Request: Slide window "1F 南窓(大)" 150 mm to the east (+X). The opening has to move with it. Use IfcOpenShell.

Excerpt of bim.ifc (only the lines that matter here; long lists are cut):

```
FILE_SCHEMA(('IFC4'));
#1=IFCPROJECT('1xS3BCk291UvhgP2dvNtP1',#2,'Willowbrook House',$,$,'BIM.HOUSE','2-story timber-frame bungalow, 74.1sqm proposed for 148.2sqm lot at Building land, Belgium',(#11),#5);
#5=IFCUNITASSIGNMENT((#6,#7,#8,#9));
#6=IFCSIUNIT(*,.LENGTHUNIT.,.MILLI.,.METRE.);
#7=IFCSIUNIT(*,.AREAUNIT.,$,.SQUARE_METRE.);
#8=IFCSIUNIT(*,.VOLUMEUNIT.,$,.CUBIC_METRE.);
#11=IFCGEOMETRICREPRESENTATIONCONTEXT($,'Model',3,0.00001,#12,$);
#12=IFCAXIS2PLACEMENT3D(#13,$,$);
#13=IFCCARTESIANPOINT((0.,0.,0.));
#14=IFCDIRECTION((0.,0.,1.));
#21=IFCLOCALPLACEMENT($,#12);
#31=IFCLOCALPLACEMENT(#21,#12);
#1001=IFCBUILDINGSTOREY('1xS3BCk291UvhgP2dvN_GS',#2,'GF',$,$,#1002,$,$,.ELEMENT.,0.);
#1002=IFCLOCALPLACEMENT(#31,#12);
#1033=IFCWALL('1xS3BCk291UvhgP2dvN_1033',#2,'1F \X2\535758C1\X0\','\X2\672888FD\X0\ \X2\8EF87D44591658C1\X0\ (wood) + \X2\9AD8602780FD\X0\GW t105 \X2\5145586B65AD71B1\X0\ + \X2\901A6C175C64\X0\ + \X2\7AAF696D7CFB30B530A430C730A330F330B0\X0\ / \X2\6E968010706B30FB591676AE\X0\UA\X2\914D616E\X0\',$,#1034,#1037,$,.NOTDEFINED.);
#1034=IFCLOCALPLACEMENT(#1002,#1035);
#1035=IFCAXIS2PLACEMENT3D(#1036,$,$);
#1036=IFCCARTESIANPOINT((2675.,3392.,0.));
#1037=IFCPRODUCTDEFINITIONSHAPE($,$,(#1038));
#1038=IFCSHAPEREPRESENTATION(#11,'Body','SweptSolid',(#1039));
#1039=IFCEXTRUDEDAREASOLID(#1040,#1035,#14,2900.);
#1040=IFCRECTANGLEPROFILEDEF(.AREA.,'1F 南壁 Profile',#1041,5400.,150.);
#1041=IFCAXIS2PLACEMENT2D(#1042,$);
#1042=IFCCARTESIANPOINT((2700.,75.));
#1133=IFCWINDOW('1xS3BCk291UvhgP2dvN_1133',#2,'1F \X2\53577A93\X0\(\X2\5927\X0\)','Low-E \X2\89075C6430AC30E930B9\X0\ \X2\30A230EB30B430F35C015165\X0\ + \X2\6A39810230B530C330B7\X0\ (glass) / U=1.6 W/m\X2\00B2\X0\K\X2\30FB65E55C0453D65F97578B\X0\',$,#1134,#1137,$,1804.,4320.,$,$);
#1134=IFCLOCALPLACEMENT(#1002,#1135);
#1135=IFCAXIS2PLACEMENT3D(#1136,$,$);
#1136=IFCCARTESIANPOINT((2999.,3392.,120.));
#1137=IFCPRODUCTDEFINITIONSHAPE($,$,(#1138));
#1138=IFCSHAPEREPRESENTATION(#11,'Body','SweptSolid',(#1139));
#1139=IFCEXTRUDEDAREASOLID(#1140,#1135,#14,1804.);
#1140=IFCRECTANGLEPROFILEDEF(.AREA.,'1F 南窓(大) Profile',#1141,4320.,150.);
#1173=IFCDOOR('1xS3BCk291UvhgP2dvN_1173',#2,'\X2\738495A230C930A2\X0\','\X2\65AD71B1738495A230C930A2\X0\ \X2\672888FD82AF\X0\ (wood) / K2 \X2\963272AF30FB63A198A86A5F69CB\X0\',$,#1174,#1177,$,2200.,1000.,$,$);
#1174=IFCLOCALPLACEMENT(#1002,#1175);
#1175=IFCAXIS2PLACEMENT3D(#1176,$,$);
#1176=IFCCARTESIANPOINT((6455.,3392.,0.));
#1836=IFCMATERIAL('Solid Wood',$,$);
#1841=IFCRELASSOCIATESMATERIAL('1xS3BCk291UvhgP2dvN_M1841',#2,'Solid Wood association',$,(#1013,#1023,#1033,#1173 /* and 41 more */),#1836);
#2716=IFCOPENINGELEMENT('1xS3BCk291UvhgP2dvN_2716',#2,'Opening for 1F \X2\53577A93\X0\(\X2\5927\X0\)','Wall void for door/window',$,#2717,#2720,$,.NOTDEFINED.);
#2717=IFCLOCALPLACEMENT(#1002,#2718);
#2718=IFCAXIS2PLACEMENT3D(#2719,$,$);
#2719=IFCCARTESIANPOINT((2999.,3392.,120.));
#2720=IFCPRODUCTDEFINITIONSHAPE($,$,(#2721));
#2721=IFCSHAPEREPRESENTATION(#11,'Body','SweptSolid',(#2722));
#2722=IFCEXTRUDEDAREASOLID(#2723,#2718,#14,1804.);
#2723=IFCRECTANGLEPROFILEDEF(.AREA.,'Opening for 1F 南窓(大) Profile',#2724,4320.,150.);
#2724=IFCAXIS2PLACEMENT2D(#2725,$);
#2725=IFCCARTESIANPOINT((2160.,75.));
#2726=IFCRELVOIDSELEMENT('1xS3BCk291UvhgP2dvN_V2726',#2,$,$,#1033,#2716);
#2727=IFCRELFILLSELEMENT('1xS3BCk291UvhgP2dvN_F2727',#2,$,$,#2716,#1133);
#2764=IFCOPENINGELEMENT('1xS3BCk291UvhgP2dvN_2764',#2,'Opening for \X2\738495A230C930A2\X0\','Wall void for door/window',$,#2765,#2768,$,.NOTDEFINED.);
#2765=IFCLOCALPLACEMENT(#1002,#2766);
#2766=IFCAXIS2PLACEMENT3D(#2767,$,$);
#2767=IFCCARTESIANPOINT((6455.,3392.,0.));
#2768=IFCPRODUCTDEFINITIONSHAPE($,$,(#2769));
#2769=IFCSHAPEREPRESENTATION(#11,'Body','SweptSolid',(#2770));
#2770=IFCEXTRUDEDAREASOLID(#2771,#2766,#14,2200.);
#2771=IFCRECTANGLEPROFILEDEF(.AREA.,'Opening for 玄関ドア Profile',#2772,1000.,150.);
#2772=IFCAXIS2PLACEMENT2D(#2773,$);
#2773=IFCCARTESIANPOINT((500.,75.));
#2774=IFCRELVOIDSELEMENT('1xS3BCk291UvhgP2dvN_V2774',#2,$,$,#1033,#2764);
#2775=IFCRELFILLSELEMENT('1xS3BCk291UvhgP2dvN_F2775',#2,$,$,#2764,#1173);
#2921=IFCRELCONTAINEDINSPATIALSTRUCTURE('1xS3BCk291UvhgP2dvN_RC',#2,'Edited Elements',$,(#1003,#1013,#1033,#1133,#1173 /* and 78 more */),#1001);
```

```python
import ifcopenshell
import ifcopenshell.api.geometry
import ifcopenshell.util.placement
import ifcopenshell.util.unit

model = ifcopenshell.open("bim.ifc")
unit_scale = ifcopenshell.util.unit.calculate_unit_scale(model)

window = model.by_guid("1xS3BCk291UvhgP2dvN_1133")
opening = window.FillsVoids[0].RelatingOpeningElement
wall = opening.VoidsElements[0].RelatingBuildingElement

wall_matrix = ifcopenshell.util.placement.get_local_placement(wall.ObjectPlacement)
shift = wall_matrix[:3, 0] * 0.15 / unit_scale
before = ifcopenshell.util.placement.get_local_placement(window.ObjectPlacement)[:3, 3].copy()

# The window is not placed relative to its opening, so move both.
for product in (opening, window):
    matrix = ifcopenshell.util.placement.get_local_placement(product.ObjectPlacement)
    matrix[:3, 3] += shift
    ifcopenshell.api.geometry.edit_object_placement(model, product=product, matrix=matrix, is_si=False)

after = ifcopenshell.util.placement.get_local_placement(window.ObjectPlacement)[:3, 3]
print("window moved by", (after - before).round(3) + 0.0)

model.write("bim_rev.ifc")
```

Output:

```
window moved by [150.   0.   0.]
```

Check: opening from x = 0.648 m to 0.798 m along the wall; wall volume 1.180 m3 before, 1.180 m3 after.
